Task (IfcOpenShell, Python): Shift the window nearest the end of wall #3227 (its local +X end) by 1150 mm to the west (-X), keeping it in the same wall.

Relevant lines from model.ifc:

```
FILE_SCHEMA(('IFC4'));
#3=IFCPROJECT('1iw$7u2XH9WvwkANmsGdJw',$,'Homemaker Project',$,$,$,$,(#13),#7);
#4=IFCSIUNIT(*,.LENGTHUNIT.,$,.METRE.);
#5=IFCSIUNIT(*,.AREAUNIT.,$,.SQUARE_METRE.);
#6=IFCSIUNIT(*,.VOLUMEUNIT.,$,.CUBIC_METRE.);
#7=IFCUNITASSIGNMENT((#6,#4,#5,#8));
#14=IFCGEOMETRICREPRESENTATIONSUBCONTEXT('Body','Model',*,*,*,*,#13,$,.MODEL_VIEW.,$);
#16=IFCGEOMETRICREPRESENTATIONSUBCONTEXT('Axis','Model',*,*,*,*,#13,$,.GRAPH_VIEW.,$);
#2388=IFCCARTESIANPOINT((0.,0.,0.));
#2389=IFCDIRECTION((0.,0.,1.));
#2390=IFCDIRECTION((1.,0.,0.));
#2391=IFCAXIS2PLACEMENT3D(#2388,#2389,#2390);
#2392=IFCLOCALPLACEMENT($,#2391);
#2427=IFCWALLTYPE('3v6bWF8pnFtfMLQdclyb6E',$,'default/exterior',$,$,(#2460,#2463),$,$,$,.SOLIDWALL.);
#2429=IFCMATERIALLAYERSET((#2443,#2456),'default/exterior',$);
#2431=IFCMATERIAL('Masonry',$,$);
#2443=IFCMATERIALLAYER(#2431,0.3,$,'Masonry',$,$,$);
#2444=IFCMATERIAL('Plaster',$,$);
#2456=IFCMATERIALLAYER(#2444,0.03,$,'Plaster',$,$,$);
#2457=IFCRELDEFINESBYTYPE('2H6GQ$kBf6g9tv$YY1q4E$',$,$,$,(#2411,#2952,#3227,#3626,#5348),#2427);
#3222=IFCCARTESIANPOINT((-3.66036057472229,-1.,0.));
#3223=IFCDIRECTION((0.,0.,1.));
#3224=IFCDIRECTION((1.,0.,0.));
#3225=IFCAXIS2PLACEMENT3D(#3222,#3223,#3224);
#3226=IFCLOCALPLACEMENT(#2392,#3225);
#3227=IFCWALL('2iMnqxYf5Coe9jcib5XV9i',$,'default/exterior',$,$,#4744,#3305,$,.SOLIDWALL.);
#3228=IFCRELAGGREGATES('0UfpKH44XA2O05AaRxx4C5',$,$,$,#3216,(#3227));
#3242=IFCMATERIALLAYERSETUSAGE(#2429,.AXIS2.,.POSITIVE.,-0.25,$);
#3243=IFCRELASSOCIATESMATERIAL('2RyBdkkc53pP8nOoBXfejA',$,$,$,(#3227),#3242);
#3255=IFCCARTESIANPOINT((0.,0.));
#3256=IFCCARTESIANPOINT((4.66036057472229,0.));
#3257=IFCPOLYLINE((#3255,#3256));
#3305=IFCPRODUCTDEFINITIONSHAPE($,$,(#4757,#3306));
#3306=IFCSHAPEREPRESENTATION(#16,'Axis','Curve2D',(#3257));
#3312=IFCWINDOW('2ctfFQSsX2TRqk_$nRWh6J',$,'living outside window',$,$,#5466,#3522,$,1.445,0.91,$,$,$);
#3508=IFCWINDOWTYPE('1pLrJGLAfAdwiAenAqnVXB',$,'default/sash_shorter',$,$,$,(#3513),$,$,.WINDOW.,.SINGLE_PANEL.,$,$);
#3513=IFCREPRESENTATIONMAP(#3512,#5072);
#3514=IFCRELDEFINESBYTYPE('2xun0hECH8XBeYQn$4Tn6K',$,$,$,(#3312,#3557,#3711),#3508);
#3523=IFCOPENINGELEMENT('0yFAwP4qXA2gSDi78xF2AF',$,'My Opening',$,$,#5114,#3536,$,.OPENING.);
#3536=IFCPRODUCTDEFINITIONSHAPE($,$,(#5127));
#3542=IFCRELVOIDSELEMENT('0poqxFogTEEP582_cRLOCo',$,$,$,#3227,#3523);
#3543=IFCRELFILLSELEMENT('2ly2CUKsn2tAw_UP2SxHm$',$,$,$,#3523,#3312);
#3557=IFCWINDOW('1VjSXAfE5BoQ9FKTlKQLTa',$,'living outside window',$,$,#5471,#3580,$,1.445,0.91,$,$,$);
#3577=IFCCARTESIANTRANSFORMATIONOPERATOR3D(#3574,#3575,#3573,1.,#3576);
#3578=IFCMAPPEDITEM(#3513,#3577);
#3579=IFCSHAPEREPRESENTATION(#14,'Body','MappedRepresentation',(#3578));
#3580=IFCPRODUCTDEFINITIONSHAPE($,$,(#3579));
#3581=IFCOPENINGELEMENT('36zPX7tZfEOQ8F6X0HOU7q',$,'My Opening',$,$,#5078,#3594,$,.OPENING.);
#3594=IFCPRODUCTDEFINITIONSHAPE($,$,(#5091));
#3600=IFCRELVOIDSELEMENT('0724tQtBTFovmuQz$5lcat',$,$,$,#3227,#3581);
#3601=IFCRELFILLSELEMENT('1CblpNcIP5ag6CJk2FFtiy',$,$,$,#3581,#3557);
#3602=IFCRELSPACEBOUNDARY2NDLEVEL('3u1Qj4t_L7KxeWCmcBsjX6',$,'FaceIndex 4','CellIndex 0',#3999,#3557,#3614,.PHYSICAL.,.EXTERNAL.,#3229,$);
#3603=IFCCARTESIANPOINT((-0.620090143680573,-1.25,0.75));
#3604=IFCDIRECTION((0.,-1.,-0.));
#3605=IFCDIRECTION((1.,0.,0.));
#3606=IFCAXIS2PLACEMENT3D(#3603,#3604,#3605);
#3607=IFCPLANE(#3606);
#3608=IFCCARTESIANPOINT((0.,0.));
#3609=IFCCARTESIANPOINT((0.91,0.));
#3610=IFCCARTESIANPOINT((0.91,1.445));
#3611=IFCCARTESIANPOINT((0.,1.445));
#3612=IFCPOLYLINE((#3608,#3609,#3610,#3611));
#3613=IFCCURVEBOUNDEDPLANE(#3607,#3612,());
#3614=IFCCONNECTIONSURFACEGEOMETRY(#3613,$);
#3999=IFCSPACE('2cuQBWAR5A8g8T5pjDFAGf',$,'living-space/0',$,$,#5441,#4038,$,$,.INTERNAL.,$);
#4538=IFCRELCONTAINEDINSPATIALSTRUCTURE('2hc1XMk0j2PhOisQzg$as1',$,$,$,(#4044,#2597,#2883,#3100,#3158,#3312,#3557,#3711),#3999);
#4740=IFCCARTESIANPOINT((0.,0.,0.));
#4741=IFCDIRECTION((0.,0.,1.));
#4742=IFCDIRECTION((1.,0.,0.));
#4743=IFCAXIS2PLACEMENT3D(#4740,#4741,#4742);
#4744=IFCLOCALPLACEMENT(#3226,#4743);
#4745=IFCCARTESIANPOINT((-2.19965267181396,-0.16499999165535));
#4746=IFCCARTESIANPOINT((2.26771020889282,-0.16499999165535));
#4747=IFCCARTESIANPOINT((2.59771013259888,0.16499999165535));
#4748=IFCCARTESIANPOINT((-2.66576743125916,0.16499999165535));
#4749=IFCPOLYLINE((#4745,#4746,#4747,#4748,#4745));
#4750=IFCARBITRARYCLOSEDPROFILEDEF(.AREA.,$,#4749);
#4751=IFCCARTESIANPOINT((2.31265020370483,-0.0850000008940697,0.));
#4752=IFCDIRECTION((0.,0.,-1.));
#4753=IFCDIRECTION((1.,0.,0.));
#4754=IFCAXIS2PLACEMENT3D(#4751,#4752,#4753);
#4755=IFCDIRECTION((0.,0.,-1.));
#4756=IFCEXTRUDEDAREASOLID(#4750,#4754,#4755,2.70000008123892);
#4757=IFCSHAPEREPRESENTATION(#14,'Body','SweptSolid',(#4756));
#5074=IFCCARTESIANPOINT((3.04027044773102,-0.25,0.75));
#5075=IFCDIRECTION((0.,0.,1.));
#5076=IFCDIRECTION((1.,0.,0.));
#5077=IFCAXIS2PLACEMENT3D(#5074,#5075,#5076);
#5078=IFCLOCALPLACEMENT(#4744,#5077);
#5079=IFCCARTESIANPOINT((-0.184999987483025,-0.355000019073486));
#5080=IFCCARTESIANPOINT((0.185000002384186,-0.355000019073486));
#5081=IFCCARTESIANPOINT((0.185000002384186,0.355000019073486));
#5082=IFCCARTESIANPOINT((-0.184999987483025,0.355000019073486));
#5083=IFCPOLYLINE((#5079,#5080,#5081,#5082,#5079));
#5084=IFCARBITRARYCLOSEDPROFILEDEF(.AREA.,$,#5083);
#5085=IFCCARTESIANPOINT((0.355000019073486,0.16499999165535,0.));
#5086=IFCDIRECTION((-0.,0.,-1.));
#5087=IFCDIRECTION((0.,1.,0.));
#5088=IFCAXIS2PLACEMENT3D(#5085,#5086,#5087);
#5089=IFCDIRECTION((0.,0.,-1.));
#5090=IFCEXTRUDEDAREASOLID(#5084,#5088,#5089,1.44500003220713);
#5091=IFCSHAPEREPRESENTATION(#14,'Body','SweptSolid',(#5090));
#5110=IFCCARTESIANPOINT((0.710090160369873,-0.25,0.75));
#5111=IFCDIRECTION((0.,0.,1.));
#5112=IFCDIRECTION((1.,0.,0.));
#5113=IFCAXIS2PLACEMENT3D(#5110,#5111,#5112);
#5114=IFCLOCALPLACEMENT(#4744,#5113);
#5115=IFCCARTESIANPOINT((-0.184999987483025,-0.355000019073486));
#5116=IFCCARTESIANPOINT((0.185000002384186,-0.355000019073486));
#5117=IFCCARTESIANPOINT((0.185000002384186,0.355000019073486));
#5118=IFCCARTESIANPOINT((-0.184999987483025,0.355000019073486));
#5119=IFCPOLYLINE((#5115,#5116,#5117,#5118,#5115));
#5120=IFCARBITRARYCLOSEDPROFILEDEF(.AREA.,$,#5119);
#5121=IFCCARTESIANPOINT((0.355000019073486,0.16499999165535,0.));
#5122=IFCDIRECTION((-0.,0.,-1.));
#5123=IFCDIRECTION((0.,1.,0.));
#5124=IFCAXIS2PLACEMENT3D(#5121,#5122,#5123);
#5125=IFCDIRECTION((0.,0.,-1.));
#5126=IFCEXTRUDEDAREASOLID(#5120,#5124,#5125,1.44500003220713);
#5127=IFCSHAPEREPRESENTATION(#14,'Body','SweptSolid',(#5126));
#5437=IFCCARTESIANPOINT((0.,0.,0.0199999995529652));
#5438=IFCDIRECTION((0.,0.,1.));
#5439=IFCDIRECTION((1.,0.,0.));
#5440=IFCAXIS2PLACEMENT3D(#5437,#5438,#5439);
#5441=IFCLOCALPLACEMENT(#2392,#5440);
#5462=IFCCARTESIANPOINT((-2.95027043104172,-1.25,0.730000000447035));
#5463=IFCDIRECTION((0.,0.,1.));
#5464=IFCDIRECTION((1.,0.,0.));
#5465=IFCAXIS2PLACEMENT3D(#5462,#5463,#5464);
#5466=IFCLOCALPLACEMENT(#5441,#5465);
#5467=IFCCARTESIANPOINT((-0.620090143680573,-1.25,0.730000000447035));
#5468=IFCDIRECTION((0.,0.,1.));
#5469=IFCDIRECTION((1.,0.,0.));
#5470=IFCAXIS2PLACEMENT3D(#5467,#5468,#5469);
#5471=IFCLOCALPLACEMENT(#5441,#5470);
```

```python
import numpy as np
import ifcopenshell
import ifcopenshell.api.geometry
import ifcopenshell.util.placement
import ifcopenshell.util.unit

model = ifcopenshell.open("model.ifc")
unit_scale = ifcopenshell.util.unit.calculate_unit_scale(model)

window = model.by_guid("1VjSXAfE5BoQ9FKTlKQLTa")
opening = window.FillsVoids[0].RelatingOpeningElement
wall = opening.VoidsElements[0].RelatingBuildingElement

wall_matrix = ifcopenshell.util.placement.get_local_placement(wall.ObjectPlacement)
shift = wall_matrix[:3, 0] * -1.15 / unit_scale
before = ifcopenshell.util.placement.get_local_placement(window.ObjectPlacement)[:3, 3].copy()

# The window is not placed relative to its opening, so move both.
for product in (opening, window):
    matrix = ifcopenshell.util.placement.get_local_placement(product.ObjectPlacement)
    matrix[:3, 3] += shift
    ifcopenshell.api.geometry.edit_object_placement(model, product=product, matrix=matrix, is_si=False)

# Space boundary surfaces are stored in each space's coordinates; move them too.
for rel in window.ProvidesBoundaries:
    if not rel.ConnectionGeometry:
        continue
    surface = rel.ConnectionGeometry.SurfaceOnRelatingElement.BasisSurface
    space_matrix = ifcopenshell.util.placement.get_local_placement(rel.RelatingSpace.ObjectPlacement)
    point = np.array(surface.Position.Location.Coordinates) + space_matrix[:3, :3].T @ shift
    surface.Position = model.createIfcAxis2Placement3D(
        model.createIfcCartesianPoint(point.tolist()), surface.Position.Axis, surface.Position.RefDirection
    )

after = ifcopenshell.util.placement.get_local_placement(window.ObjectPlacement)[:3, 3]
print("window moved by", (after - before).round(3) + 0.0)

model.write("model_edited.ifc")
```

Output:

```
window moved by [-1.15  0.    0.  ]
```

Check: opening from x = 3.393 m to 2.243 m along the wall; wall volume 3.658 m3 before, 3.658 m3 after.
